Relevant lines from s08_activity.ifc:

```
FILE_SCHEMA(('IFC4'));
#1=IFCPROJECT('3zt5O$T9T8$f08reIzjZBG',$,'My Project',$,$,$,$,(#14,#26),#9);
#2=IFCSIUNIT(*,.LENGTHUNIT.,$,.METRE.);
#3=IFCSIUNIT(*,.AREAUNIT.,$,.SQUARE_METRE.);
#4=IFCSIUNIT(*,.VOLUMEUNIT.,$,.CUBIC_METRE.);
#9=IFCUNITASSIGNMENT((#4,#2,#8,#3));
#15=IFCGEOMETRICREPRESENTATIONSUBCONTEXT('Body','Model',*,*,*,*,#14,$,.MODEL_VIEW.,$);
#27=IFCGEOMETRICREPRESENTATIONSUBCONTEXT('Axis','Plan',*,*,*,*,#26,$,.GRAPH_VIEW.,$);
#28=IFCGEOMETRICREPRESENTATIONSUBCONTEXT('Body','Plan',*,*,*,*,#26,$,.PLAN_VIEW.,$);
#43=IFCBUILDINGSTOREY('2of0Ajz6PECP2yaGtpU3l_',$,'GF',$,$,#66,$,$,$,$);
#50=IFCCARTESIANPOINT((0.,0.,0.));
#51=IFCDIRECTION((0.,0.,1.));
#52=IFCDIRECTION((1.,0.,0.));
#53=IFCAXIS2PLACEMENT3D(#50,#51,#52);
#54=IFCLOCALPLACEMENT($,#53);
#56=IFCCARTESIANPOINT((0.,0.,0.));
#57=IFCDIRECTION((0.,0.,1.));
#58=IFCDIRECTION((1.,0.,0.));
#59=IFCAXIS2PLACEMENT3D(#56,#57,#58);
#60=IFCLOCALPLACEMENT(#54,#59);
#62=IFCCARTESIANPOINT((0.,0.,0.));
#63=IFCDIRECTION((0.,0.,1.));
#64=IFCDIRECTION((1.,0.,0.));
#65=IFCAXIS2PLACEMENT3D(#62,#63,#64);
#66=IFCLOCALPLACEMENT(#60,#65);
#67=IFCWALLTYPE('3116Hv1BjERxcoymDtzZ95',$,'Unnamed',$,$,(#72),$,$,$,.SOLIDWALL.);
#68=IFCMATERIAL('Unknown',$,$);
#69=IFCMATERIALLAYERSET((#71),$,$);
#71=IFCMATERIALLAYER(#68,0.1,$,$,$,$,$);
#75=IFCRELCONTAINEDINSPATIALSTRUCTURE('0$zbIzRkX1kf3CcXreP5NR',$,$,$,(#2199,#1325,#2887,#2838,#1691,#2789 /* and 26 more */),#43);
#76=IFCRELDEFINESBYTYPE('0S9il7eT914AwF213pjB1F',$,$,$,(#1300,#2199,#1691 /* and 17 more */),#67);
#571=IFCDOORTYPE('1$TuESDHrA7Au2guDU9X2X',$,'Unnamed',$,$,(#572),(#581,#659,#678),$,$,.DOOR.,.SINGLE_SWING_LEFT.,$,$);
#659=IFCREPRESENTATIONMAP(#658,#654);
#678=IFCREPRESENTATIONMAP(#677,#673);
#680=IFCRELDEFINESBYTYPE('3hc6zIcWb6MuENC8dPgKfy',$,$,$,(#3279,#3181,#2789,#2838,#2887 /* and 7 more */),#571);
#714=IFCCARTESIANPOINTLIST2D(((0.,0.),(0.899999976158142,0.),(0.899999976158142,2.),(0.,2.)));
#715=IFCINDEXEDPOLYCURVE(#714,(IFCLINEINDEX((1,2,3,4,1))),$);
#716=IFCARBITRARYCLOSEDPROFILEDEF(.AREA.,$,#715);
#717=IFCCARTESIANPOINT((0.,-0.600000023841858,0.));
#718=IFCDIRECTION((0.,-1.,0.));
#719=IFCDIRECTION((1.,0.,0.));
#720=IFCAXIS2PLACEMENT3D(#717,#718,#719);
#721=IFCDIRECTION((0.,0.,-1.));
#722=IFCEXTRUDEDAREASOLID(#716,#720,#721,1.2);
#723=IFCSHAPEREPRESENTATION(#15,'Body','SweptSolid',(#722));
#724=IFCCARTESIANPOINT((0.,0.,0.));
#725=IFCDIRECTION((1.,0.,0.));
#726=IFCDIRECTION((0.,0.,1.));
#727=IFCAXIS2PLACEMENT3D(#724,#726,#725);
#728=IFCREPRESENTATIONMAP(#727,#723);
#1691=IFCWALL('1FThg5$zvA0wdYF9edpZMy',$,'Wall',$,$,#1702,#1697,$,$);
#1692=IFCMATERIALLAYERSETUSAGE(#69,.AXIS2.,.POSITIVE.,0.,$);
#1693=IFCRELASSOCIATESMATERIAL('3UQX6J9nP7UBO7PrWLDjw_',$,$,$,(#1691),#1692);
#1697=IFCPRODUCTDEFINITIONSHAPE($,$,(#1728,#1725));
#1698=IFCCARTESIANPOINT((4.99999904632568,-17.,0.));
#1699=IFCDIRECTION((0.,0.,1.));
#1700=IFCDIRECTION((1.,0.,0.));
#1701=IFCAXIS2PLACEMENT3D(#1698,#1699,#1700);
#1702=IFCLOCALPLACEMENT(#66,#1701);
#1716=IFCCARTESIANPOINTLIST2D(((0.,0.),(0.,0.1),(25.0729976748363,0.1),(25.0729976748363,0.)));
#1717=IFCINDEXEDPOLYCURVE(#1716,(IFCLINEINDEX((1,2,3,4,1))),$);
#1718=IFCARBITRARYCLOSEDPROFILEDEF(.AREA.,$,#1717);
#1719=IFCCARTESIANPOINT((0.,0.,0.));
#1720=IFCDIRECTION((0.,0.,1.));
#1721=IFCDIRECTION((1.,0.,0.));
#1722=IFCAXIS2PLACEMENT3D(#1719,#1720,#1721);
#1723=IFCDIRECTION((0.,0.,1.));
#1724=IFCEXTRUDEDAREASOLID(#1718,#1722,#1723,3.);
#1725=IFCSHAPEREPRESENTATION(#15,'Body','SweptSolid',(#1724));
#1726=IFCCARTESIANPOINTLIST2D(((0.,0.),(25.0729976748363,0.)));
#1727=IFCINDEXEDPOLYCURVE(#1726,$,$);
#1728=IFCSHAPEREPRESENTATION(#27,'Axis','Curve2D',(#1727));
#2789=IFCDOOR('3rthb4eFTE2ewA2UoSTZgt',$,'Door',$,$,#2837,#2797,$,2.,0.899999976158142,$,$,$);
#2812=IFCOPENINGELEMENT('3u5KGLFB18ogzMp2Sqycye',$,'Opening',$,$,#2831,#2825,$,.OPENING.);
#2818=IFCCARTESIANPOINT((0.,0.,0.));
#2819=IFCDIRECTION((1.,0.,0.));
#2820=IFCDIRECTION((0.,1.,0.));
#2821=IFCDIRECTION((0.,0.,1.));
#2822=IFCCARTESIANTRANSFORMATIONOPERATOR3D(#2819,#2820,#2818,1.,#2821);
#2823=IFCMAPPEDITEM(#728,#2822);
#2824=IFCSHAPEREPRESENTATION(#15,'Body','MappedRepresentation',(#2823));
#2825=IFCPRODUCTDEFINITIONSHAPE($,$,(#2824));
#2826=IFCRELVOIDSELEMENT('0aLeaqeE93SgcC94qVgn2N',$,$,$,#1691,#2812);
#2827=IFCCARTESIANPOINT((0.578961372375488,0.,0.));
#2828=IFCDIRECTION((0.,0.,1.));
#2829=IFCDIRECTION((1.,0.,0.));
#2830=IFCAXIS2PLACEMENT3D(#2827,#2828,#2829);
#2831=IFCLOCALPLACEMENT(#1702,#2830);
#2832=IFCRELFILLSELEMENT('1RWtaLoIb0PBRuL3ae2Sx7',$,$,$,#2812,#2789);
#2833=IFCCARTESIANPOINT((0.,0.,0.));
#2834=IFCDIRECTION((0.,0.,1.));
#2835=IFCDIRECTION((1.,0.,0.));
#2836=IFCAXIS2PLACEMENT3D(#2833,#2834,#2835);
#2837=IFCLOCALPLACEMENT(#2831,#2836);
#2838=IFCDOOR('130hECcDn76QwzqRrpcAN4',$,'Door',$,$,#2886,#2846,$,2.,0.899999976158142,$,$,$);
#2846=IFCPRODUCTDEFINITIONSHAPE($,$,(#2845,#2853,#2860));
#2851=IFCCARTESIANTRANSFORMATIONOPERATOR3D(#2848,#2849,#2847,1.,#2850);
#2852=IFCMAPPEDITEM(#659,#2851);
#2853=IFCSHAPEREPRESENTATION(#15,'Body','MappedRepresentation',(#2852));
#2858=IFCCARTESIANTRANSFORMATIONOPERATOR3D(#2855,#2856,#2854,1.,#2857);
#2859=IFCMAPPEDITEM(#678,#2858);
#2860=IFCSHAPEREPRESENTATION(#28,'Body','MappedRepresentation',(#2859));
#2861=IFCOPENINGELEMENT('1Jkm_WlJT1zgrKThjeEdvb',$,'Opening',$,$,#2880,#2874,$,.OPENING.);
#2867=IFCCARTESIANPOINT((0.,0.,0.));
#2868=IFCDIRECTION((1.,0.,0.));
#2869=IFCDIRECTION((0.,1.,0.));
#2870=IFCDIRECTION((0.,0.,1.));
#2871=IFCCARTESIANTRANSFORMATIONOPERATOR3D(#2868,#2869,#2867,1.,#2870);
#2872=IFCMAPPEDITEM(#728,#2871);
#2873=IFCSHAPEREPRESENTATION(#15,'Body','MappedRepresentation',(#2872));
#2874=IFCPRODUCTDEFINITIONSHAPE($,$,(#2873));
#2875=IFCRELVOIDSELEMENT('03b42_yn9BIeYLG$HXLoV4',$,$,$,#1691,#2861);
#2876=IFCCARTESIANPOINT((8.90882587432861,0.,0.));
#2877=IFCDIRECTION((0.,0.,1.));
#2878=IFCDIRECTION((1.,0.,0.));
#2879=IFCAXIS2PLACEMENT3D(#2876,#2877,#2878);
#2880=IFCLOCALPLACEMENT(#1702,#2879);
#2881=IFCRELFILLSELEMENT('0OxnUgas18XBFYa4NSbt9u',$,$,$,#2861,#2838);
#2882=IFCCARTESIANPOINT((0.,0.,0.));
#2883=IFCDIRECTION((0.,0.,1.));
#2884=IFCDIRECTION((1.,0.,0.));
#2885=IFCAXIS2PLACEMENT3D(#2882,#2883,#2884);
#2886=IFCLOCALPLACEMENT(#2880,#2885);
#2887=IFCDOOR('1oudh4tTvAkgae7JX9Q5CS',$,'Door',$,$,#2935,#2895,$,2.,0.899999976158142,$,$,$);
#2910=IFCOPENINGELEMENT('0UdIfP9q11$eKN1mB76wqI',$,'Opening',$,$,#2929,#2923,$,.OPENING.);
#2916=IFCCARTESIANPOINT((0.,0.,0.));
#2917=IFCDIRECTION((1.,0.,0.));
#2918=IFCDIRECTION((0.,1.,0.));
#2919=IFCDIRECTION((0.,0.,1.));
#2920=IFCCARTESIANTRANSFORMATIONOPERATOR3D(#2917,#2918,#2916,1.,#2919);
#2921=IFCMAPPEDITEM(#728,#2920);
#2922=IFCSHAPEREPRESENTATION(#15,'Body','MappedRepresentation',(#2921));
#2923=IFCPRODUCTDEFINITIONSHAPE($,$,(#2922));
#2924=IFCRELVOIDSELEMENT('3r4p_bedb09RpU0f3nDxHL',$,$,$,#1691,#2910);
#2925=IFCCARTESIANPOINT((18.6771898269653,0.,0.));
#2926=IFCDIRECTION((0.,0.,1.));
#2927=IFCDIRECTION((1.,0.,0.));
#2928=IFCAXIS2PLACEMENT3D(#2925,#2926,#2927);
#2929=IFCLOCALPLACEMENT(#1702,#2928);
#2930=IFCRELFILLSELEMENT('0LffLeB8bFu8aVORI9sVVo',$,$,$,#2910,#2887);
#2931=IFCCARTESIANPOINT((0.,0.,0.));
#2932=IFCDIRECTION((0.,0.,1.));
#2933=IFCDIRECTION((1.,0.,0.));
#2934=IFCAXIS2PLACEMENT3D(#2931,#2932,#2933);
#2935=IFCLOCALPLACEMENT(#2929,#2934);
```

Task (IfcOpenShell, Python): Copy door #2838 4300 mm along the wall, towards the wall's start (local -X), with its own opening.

```python
import ifcopenshell
import ifcopenshell.api.feature
import ifcopenshell.api.geometry
import ifcopenshell.api.root
import ifcopenshell.geom
import ifcopenshell.util.element
import ifcopenshell.util.placement
import ifcopenshell.util.shape
import ifcopenshell.util.unit

model = ifcopenshell.open("s08_activity.ifc")
unit_scale = ifcopenshell.util.unit.calculate_unit_scale(model)
settings = ifcopenshell.geom.settings()


def volume(element):
    """Net volume in cubic metres, openings subtracted."""
    shape = ifcopenshell.geom.create_shape(settings, element)
    return ifcopenshell.util.shape.get_volume(shape.geometry)


door = model.by_id(2838)
opening = door.FillsVoids[0].RelatingOpeningElement
wall = opening.VoidsElements[0].RelatingBuildingElement
before = volume(wall)
shift = ifcopenshell.util.placement.get_local_placement(wall.ObjectPlacement)[:3, 0] * -4.3 / unit_scale

# copy_class copies the void relationship, type, container and properties, but no geometry.
new_opening = ifcopenshell.api.root.copy_class(model, product=opening)
new_opening.Representation = ifcopenshell.util.element.copy_deep(
    model, opening.Representation, exclude=["IfcGeometricRepresentationContext", "IfcRepresentationMap"]
)
new_door = ifcopenshell.api.root.copy_class(model, product=door)
new_door.Representation = ifcopenshell.util.element.copy_deep(
    model, door.Representation, exclude=["IfcGeometricRepresentationContext", "IfcRepresentationMap"]
)
ifcopenshell.api.feature.add_filling(model, opening=new_opening, element=new_door)

for old, new in ((opening, new_opening), (door, new_door)):
    matrix = ifcopenshell.util.placement.get_local_placement(old.ObjectPlacement)
    matrix[:3, 3] += shift
    ifcopenshell.api.geometry.edit_object_placement(model, product=new, matrix=matrix, is_si=False)

after = volume(wall)

print(f"wall volume {before:.3f} -> {after:.3f} m3")

model.write("s08_activity-out.ifc")
```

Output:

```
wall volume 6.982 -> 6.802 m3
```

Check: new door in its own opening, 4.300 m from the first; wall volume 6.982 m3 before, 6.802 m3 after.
